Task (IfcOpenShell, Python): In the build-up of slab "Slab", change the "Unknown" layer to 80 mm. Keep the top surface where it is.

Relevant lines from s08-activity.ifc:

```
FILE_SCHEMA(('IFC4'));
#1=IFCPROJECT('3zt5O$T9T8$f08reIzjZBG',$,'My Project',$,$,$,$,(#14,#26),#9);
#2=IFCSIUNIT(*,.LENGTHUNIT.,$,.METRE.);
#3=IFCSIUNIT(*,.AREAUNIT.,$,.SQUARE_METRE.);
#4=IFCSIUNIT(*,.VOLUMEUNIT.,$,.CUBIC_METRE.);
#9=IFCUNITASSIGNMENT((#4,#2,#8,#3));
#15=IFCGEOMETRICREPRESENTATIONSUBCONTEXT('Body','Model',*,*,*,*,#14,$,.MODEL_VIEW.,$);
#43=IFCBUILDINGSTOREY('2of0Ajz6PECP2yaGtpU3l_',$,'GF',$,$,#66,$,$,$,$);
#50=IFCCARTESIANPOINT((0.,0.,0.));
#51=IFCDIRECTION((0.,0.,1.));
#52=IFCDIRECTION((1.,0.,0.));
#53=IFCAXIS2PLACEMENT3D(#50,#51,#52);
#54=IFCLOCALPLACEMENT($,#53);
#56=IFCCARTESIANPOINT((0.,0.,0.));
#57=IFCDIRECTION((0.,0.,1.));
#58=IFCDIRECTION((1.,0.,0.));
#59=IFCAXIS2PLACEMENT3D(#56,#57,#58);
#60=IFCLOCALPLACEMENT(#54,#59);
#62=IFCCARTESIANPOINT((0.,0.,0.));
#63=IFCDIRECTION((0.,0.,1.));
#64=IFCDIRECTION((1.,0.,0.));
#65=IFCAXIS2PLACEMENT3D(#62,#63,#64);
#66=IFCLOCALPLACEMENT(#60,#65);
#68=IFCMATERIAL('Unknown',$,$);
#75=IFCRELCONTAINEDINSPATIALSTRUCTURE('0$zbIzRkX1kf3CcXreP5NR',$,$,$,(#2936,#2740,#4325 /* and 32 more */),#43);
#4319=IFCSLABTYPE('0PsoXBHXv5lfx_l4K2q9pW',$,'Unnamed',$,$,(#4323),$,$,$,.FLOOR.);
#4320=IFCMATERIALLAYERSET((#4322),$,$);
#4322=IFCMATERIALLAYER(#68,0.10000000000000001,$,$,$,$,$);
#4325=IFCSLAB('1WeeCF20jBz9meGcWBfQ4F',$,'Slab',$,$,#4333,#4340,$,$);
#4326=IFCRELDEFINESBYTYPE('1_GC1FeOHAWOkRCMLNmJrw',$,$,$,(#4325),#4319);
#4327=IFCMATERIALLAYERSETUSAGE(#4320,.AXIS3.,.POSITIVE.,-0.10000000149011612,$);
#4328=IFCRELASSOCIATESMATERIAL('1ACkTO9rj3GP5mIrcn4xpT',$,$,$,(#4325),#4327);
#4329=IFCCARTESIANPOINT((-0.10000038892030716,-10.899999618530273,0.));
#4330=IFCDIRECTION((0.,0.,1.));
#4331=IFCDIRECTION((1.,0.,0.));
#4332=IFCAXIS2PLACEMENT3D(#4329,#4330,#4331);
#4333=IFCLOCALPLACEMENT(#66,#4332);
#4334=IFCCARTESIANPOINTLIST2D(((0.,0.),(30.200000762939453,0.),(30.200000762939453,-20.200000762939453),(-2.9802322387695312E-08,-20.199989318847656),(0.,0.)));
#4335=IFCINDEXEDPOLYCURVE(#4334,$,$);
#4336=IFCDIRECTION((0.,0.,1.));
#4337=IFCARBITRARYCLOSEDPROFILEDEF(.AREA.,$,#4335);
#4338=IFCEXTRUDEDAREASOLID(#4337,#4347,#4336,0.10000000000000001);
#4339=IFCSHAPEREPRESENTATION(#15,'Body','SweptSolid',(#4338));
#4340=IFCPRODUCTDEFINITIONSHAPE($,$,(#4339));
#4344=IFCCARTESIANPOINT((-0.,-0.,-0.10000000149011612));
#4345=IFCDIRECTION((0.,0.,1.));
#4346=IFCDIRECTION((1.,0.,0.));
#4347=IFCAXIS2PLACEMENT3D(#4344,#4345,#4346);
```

```python
import ifcopenshell
import ifcopenshell.util.element
import ifcopenshell.util.representation

model = ifcopenshell.open("s08-activity.ifc")

layer_set = model.by_id(4320)
layer = next(l for l in layer_set.MaterialLayers if l.Material and l.Material.Name == "Unknown")
change = 0.08 - layer.LayerThickness
layer.LayerThickness += change

# Geometry does not follow the layer set by itself.
slabs = [e for e in ifcopenshell.util.element.get_elements_by_material(model, layer_set) if e.is_a("IfcSlab")]
for slab in sorted(slabs, key=lambda e: e.id()):
    body = ifcopenshell.util.representation.get_representation(slab, "Model", "Body")
    solid = body.Items[0]
    old_depth = solid.Depth
    solid.Depth += change
    # Extruded upwards: lower the start of the extrusion so the top stays.
    x, y, z = solid.Position.Location.Coordinates
    solid.Position.Location = model.createIfcCartesianPoint((x, y, z - change))
    print(slab.id(), f"{old_depth:g} -> {solid.Depth:g}")

# The layers are counted up from the underside, which has moved.
for usage in {ifcopenshell.util.element.get_material(slab) for slab in slabs}:
    usage.OffsetFromReferenceLine -= change

model.write("s08-activity_rev.ifc")
```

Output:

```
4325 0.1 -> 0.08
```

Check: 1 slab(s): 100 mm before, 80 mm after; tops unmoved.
